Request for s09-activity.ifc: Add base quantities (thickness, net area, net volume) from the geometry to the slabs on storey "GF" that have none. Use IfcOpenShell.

First a look at what the model holds.

```python
import ifcopenshell
import ifcopenshell.util.element
import ifcopenshell.util.unit

model = ifcopenshell.open("s09-activity.ifc")
print(model.schema)
for unit_type in ("LENGTHUNIT", "AREAUNIT", "VOLUMEUNIT"):
    print(unit_type, ifcopenshell.util.unit.calculate_unit_scale(model, unit_type))
storey = next(s for s in model.by_type("IfcBuildingStorey") if s.Name == "GF")
slabs = [e for e in ifcopenshell.util.element.get_decomposition(storey) if e.is_a("IfcSlab")]
for e in sorted(slabs, key=lambda e: e.id()):
    print(e.id(), e.is_a(), e.Name, list(ifcopenshell.util.element.get_psets(e, qtos_only=True)), sep=" | ")
```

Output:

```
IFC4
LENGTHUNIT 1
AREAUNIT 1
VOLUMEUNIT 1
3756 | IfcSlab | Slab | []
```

```python
import ifcopenshell
import ifcopenshell.api.pset
import ifcopenshell.geom
import ifcopenshell.util.element
import ifcopenshell.util.shape
import ifcopenshell.util.unit

model = ifcopenshell.open("s09-activity.ifc")
unit_scale = ifcopenshell.util.unit.calculate_unit_scale(model)
area_scale = ifcopenshell.util.unit.calculate_unit_scale(model, "AREAUNIT")
volume_scale = ifcopenshell.util.unit.calculate_unit_scale(model, "VOLUMEUNIT")
settings = ifcopenshell.geom.settings()

storey = next(s for s in model.by_type("IfcBuildingStorey") if s.Name == "GF")
slabs = [e for e in ifcopenshell.util.element.get_decomposition(storey) if e.is_a("IfcSlab")]

for e in sorted(slabs, key=lambda e: e.id()):
    if ifcopenshell.util.element.get_psets(e, qtos_only=True, should_inherit=False):
        continue
    # Geometry comes back in metres, in the element's own axes.
    shape = ifcopenshell.geom.create_shape(settings, e)
    values = {
        "Width": ifcopenshell.util.shape.get_z(shape.geometry) / unit_scale,
        "NetArea": ifcopenshell.util.shape.get_footprint_area(shape.geometry) / area_scale,
        "NetVolume": ifcopenshell.util.shape.get_volume(shape.geometry) / volume_scale,
    }
    qto = ifcopenshell.api.pset.add_qto(model, product=e, name="Qto_SlabBaseQuantities")
    ifcopenshell.api.pset.edit_qto(model, qto=qto, properties=values)
    print(e.id(), {k: round(v, 3) for k, v in values.items()})

model.write("s09-activity_updated.ifc")
```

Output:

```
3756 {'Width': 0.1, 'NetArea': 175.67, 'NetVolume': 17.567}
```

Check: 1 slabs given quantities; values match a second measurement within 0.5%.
